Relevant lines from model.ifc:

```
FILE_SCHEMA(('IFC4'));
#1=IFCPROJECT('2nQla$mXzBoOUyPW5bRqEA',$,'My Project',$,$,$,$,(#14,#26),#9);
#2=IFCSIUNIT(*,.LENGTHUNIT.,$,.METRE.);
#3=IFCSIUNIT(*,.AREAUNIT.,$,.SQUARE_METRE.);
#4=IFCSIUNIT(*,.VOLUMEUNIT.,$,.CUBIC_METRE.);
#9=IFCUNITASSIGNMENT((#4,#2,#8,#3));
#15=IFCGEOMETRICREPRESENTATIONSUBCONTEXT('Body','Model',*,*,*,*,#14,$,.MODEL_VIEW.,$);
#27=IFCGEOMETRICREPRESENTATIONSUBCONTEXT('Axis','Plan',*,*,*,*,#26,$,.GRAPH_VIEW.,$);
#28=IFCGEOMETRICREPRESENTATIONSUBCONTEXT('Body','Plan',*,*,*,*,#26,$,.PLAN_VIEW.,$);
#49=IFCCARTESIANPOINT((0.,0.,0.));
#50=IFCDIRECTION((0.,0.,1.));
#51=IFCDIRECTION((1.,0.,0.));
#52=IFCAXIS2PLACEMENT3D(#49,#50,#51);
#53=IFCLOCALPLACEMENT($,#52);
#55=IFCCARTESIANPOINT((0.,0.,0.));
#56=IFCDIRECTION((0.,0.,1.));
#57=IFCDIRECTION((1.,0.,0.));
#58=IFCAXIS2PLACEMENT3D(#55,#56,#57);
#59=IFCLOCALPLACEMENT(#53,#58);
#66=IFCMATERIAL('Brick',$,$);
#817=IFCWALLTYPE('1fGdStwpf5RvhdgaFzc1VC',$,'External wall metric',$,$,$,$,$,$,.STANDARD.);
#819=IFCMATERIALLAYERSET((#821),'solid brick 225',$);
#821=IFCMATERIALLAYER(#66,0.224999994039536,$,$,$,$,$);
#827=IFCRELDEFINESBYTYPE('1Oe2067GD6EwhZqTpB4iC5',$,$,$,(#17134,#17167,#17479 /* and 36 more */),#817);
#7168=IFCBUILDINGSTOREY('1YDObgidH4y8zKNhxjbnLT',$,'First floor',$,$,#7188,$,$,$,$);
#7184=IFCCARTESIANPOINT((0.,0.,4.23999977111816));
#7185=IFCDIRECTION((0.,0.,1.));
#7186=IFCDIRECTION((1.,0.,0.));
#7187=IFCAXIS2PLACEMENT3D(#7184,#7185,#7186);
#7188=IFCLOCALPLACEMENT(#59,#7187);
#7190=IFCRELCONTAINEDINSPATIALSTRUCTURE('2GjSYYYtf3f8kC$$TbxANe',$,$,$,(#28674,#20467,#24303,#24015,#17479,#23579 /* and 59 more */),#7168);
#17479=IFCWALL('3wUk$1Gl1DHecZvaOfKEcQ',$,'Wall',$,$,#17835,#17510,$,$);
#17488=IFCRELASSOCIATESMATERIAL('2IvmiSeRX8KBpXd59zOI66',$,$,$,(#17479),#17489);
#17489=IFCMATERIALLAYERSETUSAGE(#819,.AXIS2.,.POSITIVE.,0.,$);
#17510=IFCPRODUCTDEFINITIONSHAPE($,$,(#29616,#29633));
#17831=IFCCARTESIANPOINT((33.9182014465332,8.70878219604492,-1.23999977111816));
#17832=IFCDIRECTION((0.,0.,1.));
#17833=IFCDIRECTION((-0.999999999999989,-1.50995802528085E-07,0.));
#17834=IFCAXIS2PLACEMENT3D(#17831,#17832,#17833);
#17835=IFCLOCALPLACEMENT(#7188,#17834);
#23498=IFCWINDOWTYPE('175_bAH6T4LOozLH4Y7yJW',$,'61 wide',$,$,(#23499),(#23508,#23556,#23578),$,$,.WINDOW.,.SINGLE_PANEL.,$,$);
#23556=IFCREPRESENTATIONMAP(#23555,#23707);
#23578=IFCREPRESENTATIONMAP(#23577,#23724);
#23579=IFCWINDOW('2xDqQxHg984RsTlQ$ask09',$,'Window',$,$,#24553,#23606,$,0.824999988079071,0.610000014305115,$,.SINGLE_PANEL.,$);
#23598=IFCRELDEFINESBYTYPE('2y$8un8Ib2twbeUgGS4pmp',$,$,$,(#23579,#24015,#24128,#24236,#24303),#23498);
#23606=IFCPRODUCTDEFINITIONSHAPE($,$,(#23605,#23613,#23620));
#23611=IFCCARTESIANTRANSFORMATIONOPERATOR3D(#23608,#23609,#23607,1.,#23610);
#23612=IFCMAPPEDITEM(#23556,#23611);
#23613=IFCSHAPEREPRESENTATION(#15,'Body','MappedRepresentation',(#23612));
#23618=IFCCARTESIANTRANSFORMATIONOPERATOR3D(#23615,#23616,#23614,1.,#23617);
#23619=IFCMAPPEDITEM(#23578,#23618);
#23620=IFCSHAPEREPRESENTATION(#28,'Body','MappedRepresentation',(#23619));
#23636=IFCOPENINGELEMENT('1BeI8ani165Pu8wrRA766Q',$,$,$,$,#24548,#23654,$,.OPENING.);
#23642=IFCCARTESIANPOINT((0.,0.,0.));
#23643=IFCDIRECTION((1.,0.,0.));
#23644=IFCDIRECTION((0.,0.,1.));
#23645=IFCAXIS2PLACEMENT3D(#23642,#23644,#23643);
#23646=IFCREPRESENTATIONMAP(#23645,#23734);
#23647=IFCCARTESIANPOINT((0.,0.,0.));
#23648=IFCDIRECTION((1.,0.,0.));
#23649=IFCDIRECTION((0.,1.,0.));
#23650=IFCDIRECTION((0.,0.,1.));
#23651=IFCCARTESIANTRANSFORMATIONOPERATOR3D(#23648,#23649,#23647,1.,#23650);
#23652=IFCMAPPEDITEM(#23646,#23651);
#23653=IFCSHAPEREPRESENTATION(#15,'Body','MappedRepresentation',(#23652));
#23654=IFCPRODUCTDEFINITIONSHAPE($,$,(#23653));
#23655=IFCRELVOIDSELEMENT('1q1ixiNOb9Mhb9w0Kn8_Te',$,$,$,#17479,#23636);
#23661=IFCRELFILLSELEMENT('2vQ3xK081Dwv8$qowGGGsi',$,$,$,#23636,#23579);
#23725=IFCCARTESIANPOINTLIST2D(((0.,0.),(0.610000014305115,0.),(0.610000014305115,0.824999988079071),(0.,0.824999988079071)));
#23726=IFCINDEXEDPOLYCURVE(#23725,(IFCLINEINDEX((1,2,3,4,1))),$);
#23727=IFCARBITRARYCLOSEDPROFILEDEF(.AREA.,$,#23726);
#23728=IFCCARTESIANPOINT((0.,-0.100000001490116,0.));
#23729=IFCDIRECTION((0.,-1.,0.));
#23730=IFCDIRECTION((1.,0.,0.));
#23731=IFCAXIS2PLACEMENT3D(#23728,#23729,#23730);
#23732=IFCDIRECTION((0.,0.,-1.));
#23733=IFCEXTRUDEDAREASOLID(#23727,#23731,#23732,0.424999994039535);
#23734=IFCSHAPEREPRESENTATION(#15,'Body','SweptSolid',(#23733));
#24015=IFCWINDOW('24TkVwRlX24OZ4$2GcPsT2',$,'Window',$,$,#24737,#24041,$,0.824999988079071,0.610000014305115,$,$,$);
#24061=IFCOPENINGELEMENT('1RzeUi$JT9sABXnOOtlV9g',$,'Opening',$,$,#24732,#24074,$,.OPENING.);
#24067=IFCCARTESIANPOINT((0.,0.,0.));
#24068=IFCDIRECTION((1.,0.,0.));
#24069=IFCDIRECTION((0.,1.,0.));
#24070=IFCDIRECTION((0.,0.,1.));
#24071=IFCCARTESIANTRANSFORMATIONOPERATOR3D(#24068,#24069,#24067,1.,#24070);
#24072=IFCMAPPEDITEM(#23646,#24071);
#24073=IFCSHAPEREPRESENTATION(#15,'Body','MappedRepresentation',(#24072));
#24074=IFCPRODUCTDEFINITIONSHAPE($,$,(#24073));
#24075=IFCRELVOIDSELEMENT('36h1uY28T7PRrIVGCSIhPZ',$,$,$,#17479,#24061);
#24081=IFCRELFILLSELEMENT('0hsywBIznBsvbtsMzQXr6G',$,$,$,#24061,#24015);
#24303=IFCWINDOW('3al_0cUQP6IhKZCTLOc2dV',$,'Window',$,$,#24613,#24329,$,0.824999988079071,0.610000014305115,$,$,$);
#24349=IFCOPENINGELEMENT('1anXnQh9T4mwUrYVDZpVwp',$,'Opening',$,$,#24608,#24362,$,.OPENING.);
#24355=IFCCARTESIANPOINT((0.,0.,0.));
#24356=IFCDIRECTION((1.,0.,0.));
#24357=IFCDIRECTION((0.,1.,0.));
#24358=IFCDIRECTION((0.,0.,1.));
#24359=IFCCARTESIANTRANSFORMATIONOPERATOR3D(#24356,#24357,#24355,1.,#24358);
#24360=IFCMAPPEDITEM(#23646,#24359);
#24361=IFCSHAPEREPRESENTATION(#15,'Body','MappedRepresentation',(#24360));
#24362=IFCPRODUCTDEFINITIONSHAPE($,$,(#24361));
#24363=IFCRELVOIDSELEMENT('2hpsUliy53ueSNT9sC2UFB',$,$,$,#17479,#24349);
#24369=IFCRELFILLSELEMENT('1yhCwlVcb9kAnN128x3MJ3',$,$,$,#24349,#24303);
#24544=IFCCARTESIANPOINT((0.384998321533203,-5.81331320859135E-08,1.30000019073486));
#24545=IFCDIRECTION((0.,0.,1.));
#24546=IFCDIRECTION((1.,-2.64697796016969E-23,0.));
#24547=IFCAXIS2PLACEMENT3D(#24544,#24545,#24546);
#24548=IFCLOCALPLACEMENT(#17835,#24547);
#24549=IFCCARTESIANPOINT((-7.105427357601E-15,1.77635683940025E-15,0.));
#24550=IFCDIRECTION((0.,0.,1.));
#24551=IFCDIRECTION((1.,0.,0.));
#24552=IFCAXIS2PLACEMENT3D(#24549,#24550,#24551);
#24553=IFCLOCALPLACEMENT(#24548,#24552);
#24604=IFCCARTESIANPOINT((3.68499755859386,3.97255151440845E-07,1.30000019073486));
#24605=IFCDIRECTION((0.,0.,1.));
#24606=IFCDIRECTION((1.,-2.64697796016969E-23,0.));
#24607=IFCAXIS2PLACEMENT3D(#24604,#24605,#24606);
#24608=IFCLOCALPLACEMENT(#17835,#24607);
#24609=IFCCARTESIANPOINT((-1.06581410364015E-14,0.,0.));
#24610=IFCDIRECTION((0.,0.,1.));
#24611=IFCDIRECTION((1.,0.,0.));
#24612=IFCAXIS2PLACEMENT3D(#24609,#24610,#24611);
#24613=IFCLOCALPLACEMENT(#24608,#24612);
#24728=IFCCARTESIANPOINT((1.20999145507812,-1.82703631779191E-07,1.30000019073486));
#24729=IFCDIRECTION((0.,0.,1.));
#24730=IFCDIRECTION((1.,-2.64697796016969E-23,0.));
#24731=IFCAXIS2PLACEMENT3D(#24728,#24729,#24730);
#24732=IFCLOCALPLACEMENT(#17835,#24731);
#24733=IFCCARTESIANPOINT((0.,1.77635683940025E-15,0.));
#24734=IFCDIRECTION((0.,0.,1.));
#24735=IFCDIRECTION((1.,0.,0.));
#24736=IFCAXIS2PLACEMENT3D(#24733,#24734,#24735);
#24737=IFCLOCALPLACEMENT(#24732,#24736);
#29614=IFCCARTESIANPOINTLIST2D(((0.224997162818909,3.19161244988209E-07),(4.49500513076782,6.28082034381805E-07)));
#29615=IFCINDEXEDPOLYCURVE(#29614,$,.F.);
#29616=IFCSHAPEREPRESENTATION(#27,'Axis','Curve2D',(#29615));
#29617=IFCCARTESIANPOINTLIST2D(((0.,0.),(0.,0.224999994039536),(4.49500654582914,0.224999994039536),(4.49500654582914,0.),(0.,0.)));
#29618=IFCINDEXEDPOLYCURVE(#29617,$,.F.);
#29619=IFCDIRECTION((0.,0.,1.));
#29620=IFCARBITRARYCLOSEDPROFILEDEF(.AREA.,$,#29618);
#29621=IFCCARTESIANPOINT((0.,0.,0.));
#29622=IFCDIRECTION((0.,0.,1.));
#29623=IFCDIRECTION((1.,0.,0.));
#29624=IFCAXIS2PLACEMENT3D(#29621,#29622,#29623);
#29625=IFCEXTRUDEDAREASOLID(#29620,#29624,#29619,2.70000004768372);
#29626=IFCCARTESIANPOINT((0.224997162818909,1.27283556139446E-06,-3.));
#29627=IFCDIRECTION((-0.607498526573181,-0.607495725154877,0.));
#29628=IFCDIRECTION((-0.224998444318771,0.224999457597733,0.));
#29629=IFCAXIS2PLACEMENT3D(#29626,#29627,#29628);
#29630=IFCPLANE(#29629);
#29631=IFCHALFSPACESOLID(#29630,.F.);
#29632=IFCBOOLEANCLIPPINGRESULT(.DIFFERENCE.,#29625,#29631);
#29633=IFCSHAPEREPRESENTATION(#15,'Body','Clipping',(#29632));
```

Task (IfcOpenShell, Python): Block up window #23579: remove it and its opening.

```python
import ifcopenshell
import ifcopenshell.api.feature
import ifcopenshell.api.root
import ifcopenshell.geom
import ifcopenshell.util.shape

model = ifcopenshell.open("model.ifc")
settings = ifcopenshell.geom.settings()


def volume(element):
    """Net volume in cubic metres, openings subtracted."""
    shape = ifcopenshell.geom.create_shape(settings, element)
    return ifcopenshell.util.shape.get_volume(shape.geometry)


window = model.by_id(23579)
opening = window.FillsVoids[0].RelatingOpeningElement
wall = opening.VoidsElements[0].RelatingBuildingElement
before = volume(wall)

ifcopenshell.api.root.remove_product(model, product=window)
ifcopenshell.api.feature.remove_feature(model, feature=opening)

after = volume(wall)

print(f"wall volume {before:.3f} -> {after:.3f} m3")

model.write("model_updated.ifc")
```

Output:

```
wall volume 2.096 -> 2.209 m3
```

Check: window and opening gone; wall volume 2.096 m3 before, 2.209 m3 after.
